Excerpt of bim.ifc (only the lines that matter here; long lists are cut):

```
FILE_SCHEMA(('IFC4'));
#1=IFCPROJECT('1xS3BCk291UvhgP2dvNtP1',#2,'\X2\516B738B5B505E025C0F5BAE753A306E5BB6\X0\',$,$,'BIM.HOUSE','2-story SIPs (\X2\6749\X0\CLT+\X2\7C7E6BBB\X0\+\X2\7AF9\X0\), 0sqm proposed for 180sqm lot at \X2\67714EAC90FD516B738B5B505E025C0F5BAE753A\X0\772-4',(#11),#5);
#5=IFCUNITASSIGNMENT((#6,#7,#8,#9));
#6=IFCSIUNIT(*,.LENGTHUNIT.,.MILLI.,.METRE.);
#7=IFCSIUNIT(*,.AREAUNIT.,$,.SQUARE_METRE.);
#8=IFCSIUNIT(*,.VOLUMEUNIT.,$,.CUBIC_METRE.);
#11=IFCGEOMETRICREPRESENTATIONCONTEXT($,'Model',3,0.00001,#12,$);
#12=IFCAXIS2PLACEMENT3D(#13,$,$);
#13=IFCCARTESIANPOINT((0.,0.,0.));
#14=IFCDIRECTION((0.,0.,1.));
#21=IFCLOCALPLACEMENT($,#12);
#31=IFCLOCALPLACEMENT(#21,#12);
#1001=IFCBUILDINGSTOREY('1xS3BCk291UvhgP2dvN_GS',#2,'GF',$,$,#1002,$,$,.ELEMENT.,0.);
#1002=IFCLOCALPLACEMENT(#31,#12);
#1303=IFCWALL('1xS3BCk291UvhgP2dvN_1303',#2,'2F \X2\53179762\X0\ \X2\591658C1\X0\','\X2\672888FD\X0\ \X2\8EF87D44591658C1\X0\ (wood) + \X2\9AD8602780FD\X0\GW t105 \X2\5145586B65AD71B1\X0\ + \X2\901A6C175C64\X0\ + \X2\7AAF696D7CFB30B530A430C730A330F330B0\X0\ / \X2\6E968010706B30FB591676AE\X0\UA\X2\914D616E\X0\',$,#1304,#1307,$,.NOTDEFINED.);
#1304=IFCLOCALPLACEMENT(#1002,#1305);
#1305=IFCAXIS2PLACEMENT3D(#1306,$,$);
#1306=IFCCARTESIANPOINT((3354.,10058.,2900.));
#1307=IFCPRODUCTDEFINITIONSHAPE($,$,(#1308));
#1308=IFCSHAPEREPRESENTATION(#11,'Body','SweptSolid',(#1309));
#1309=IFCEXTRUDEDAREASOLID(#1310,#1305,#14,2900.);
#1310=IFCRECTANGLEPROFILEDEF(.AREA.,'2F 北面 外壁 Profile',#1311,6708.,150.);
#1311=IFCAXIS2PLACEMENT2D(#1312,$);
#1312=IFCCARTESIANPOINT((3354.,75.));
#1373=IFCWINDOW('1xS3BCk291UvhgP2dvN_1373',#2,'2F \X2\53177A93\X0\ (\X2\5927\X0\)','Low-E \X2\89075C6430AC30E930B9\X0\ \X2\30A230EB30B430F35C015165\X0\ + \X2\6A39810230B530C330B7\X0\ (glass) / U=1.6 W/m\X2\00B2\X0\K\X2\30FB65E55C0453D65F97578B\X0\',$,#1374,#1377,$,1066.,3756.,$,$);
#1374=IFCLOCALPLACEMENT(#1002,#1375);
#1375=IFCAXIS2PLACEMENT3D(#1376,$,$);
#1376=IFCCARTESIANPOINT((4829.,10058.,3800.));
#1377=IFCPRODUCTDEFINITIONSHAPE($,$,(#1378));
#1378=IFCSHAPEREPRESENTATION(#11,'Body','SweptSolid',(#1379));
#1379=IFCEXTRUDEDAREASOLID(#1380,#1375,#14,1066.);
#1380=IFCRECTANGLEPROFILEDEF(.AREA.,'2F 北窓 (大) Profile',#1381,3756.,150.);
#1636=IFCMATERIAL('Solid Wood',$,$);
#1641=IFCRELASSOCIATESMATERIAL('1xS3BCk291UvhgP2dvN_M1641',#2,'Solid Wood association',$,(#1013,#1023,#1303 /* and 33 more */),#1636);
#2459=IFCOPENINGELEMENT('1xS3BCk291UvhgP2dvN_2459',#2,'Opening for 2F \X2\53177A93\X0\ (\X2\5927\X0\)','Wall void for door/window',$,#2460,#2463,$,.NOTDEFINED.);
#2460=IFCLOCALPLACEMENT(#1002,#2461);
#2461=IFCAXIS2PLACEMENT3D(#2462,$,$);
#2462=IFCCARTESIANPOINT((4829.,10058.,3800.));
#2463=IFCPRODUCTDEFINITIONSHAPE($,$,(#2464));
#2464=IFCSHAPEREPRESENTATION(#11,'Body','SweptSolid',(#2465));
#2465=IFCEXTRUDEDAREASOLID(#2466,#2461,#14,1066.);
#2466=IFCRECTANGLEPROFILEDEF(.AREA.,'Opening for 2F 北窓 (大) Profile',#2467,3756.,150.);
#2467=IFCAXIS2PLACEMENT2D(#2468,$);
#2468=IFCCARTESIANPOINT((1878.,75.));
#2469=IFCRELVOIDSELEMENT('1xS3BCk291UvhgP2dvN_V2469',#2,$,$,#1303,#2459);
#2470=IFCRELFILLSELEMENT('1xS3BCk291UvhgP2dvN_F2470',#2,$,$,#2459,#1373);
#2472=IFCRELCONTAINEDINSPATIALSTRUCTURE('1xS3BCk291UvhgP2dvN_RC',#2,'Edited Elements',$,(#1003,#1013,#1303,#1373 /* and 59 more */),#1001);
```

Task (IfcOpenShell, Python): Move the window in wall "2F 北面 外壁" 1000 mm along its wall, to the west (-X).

```python
import ifcopenshell
import ifcopenshell.api.geometry
import ifcopenshell.util.placement
import ifcopenshell.util.unit

model = ifcopenshell.open("bim.ifc")
unit_scale = ifcopenshell.util.unit.calculate_unit_scale(model)

window = model.by_guid("1xS3BCk291UvhgP2dvN_1373")
opening = window.FillsVoids[0].RelatingOpeningElement
wall = opening.VoidsElements[0].RelatingBuildingElement

wall_matrix = ifcopenshell.util.placement.get_local_placement(wall.ObjectPlacement)
shift = wall_matrix[:3, 0] * -1 / unit_scale
before = ifcopenshell.util.placement.get_local_placement(window.ObjectPlacement)[:3, 3].copy()

# The window is not placed relative to its opening, so move both.
for product in (opening, window):
    matrix = ifcopenshell.util.placement.get_local_placement(product.ObjectPlacement)
    matrix[:3, 3] += shift
    ifcopenshell.api.geometry.edit_object_placement(model, product=product, matrix=matrix, is_si=False)

after = ifcopenshell.util.placement.get_local_placement(window.ObjectPlacement)[:3, 3]
print("window moved by", (after - before).round(3) + 0.0)

model.write("bim_updated.ifc")
```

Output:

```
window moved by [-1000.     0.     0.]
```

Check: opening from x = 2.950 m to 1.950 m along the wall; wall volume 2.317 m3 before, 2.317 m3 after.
